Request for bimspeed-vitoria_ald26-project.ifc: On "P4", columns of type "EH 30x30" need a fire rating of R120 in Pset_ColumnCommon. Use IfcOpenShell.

First a look at what the model holds.

```python
import ifcopenshell
import ifcopenshell.util.element

model = ifcopenshell.open("bimspeed-vitoria_ald26-project.ifc")
print(model.schema)
storey = next(s for s in model.by_type("IfcBuildingStorey") if s.Name == "P4")
columns = [e for e in ifcopenshell.util.element.get_decomposition(storey) if e.is_a("IfcColumn")]
seen = {}
for e in columns:
    element_type = ifcopenshell.util.element.get_type(e)
    key = (element_type.Name if element_type != e and element_type else None, ifcopenshell.util.element.get_pset(e, "Pset_ColumnCommon", "FireRating"))
    seen[key] = seen.get(key, 0) + 1
for (name, value), count in sorted(seen.items(), key=str):
    print(count, "x", name, "|", value)
```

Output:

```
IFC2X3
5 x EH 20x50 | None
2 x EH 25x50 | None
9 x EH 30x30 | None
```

```python
import ifcopenshell
import ifcopenshell.api.pset
import ifcopenshell.util.element

model = ifcopenshell.open("bimspeed-vitoria_ald26-project.ifc")

storey = next(s for s in model.by_type("IfcBuildingStorey") if s.Name == "P4")
columns = [e for e in ifcopenshell.util.element.get_decomposition(storey) if e.is_a("IfcColumn")]

count = 0
for e in columns:
    element_type = ifcopenshell.util.element.get_type(e)
    if element_type in (None, e) or element_type.Name != "EH 30x30":
        continue
    # add_pset returns the element's existing set when there is one.
    pset = ifcopenshell.api.pset.add_pset(model, product=e, name="Pset_ColumnCommon")
    ifcopenshell.api.pset.edit_pset(model, pset=pset, properties={"FireRating": "R120"})
    count += 1

print(count, "columns updated")

model.write("bimspeed-vitoria_ald26-project_edited.ifc")
```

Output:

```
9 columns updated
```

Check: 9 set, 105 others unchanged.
